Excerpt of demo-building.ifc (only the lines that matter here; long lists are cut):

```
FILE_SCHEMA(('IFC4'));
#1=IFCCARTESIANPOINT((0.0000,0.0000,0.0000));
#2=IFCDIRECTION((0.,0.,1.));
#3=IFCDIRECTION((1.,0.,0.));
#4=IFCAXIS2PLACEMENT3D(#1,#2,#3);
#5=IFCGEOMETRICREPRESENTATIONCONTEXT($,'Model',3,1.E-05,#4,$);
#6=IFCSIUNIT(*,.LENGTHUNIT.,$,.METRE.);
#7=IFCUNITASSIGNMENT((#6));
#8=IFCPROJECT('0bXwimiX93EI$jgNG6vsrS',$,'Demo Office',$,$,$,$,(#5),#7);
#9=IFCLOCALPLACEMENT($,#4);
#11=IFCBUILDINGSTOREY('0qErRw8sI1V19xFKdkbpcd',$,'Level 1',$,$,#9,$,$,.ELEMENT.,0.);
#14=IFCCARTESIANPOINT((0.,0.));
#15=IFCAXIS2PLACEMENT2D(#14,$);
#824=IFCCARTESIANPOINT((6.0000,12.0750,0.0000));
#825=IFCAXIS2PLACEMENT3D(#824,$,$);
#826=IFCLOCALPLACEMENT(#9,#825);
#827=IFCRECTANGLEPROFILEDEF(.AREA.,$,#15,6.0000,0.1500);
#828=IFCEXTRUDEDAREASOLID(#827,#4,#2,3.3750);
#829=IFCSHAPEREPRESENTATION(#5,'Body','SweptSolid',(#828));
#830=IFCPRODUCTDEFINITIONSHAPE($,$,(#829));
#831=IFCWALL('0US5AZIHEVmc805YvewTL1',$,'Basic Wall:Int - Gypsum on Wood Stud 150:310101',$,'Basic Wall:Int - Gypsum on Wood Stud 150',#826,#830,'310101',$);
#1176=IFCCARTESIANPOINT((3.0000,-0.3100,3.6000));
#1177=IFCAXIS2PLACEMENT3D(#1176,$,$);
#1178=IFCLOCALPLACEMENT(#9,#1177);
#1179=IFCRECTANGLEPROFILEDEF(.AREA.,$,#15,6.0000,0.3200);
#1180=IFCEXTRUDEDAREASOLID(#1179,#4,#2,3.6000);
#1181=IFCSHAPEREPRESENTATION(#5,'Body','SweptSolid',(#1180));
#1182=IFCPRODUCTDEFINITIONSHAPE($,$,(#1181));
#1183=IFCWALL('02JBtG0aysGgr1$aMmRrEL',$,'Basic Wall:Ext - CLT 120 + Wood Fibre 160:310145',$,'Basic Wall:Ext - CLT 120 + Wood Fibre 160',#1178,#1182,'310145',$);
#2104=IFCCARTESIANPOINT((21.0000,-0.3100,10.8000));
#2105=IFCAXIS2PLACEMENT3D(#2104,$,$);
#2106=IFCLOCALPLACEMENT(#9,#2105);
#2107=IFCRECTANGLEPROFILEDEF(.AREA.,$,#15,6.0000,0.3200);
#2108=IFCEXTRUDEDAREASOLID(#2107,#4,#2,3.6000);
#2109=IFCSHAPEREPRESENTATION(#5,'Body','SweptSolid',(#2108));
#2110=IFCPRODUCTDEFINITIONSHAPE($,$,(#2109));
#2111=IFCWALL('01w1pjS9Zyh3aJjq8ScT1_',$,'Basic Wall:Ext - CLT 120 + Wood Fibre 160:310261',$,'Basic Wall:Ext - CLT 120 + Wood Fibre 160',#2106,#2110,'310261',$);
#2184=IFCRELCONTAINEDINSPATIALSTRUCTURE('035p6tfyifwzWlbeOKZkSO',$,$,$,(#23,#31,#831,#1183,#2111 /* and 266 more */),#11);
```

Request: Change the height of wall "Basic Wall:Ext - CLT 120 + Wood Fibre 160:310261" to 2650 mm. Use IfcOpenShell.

```python
import ifcopenshell
import ifcopenshell.geom
import ifcopenshell.util.shape
import ifcopenshell.util.unit

model = ifcopenshell.open("demo-building.ifc")
unit_scale = ifcopenshell.util.unit.calculate_unit_scale(model)
settings = ifcopenshell.geom.settings()


def volume(element):
    """Net volume in cubic metres, openings subtracted."""
    shape = ifcopenshell.geom.create_shape(settings, element)
    return ifcopenshell.util.shape.get_volume(shape.geometry)


wall = model.by_guid("01w1pjS9Zyh3aJjq8ScT1_")
before = volume(wall)

body = next(r for r in wall.Representation.Representations if r.RepresentationIdentifier == "Body")
solid = body.Items[0]
old_height = solid.Depth
solid.Depth = 2.65 / unit_scale
after = volume(wall)

print(f"height {old_height:g} -> {solid.Depth:g}, volume {before:.3f} -> {after:.3f} m3")

model.write("demo-building_updated.ifc")
```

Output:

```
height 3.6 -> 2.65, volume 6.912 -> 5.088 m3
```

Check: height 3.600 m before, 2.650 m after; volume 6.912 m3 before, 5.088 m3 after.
